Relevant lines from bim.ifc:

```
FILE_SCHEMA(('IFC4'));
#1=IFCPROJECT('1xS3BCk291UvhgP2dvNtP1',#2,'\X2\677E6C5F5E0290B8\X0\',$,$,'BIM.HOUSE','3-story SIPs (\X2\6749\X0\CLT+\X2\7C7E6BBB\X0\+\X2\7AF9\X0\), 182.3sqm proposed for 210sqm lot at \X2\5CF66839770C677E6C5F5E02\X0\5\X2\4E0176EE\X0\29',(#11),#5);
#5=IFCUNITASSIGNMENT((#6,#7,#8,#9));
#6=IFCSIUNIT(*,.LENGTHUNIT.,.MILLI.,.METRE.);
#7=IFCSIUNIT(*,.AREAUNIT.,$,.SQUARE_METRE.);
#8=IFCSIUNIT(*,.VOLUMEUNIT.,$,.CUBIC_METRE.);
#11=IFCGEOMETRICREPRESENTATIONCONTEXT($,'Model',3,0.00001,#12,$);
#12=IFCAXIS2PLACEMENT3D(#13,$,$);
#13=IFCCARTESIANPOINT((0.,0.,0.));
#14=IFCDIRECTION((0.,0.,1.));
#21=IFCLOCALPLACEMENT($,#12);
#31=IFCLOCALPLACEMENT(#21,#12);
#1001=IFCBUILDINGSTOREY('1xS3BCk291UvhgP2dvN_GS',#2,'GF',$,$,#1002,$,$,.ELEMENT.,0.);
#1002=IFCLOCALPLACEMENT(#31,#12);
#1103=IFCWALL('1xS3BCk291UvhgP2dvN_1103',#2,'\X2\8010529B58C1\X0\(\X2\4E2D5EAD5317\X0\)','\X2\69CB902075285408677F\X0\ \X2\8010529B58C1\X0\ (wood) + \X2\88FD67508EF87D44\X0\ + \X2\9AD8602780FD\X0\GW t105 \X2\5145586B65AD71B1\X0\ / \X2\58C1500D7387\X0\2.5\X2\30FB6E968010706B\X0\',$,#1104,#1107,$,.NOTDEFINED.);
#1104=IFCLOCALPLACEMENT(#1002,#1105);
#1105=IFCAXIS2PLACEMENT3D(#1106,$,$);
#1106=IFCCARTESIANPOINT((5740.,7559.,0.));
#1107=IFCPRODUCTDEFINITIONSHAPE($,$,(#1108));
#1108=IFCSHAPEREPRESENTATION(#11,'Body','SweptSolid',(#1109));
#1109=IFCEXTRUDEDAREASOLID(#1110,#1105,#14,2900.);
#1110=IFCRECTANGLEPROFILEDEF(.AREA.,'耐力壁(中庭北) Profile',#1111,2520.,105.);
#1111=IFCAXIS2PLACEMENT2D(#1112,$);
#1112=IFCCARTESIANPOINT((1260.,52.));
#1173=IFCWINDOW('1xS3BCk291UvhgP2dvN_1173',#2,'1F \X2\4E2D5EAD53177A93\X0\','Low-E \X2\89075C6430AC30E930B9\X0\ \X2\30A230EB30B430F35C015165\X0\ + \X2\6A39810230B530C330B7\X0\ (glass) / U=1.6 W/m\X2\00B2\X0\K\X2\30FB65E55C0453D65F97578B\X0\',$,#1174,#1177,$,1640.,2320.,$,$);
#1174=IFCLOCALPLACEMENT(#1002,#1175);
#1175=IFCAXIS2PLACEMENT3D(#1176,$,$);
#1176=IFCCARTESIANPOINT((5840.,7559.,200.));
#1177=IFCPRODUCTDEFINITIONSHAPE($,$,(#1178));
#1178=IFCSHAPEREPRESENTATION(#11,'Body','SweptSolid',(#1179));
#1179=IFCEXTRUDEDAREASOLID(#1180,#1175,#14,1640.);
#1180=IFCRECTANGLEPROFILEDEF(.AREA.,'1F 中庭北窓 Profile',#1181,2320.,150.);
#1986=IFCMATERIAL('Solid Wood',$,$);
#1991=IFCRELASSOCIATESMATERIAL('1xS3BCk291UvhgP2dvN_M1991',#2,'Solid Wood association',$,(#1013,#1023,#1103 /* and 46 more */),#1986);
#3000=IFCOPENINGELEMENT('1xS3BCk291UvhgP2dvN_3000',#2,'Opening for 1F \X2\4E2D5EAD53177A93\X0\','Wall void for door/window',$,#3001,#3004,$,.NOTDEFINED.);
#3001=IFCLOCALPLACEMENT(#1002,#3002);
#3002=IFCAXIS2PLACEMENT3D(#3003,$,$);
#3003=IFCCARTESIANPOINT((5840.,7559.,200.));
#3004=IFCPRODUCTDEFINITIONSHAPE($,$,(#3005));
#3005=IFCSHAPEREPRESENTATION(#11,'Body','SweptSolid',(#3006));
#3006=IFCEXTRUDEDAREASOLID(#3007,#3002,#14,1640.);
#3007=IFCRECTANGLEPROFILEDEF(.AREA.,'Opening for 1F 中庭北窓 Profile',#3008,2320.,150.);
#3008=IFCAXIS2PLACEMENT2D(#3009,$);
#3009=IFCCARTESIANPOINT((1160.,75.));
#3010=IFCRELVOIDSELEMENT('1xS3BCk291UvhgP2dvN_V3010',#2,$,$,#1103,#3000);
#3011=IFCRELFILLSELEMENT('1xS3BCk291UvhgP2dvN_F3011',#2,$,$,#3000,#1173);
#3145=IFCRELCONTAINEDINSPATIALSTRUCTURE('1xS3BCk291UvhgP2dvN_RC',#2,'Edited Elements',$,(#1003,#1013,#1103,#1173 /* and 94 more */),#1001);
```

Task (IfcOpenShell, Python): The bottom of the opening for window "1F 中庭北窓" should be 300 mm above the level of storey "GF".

```python
import numpy as np
import ifcopenshell
import ifcopenshell.api.geometry
import ifcopenshell.geom
import ifcopenshell.util.element
import ifcopenshell.util.placement
import ifcopenshell.util.shape
import ifcopenshell.util.unit

model = ifcopenshell.open("bim.ifc")
unit_scale = ifcopenshell.util.unit.calculate_unit_scale(model)

window = model.by_guid("1xS3BCk291UvhgP2dvN_1173")
opening = window.FillsVoids[0].RelatingOpeningElement
storey = ifcopenshell.util.element.get_container(window, ifc_class="IfcBuildingStorey")
level = ifcopenshell.util.placement.get_local_placement(storey.ObjectPlacement)[2, 3]

# The opening's origin need not be at the sill, so measure its lowest point.
shape = ifcopenshell.geom.create_shape(ifcopenshell.geom.settings(), opening)
bottom = ifcopenshell.util.shape.get_shape_bottom_elevation(shape, shape.geometry) / unit_scale
dz = level + 0.3 / unit_scale - bottom

shift = np.array([0.0, 0.0, dz])
# The window is not placed relative to its opening, so move both.
for product in (opening, window):
    matrix = ifcopenshell.util.placement.get_local_placement(product.ObjectPlacement)
    matrix[:3, 3] += shift
    ifcopenshell.api.geometry.edit_object_placement(model, product=product, matrix=matrix, is_si=False)

print(f"moved by {dz * unit_scale:+.3f} m")

model.write("bim_rev.ifc")
```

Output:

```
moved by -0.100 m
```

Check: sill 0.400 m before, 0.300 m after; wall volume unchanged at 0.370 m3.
